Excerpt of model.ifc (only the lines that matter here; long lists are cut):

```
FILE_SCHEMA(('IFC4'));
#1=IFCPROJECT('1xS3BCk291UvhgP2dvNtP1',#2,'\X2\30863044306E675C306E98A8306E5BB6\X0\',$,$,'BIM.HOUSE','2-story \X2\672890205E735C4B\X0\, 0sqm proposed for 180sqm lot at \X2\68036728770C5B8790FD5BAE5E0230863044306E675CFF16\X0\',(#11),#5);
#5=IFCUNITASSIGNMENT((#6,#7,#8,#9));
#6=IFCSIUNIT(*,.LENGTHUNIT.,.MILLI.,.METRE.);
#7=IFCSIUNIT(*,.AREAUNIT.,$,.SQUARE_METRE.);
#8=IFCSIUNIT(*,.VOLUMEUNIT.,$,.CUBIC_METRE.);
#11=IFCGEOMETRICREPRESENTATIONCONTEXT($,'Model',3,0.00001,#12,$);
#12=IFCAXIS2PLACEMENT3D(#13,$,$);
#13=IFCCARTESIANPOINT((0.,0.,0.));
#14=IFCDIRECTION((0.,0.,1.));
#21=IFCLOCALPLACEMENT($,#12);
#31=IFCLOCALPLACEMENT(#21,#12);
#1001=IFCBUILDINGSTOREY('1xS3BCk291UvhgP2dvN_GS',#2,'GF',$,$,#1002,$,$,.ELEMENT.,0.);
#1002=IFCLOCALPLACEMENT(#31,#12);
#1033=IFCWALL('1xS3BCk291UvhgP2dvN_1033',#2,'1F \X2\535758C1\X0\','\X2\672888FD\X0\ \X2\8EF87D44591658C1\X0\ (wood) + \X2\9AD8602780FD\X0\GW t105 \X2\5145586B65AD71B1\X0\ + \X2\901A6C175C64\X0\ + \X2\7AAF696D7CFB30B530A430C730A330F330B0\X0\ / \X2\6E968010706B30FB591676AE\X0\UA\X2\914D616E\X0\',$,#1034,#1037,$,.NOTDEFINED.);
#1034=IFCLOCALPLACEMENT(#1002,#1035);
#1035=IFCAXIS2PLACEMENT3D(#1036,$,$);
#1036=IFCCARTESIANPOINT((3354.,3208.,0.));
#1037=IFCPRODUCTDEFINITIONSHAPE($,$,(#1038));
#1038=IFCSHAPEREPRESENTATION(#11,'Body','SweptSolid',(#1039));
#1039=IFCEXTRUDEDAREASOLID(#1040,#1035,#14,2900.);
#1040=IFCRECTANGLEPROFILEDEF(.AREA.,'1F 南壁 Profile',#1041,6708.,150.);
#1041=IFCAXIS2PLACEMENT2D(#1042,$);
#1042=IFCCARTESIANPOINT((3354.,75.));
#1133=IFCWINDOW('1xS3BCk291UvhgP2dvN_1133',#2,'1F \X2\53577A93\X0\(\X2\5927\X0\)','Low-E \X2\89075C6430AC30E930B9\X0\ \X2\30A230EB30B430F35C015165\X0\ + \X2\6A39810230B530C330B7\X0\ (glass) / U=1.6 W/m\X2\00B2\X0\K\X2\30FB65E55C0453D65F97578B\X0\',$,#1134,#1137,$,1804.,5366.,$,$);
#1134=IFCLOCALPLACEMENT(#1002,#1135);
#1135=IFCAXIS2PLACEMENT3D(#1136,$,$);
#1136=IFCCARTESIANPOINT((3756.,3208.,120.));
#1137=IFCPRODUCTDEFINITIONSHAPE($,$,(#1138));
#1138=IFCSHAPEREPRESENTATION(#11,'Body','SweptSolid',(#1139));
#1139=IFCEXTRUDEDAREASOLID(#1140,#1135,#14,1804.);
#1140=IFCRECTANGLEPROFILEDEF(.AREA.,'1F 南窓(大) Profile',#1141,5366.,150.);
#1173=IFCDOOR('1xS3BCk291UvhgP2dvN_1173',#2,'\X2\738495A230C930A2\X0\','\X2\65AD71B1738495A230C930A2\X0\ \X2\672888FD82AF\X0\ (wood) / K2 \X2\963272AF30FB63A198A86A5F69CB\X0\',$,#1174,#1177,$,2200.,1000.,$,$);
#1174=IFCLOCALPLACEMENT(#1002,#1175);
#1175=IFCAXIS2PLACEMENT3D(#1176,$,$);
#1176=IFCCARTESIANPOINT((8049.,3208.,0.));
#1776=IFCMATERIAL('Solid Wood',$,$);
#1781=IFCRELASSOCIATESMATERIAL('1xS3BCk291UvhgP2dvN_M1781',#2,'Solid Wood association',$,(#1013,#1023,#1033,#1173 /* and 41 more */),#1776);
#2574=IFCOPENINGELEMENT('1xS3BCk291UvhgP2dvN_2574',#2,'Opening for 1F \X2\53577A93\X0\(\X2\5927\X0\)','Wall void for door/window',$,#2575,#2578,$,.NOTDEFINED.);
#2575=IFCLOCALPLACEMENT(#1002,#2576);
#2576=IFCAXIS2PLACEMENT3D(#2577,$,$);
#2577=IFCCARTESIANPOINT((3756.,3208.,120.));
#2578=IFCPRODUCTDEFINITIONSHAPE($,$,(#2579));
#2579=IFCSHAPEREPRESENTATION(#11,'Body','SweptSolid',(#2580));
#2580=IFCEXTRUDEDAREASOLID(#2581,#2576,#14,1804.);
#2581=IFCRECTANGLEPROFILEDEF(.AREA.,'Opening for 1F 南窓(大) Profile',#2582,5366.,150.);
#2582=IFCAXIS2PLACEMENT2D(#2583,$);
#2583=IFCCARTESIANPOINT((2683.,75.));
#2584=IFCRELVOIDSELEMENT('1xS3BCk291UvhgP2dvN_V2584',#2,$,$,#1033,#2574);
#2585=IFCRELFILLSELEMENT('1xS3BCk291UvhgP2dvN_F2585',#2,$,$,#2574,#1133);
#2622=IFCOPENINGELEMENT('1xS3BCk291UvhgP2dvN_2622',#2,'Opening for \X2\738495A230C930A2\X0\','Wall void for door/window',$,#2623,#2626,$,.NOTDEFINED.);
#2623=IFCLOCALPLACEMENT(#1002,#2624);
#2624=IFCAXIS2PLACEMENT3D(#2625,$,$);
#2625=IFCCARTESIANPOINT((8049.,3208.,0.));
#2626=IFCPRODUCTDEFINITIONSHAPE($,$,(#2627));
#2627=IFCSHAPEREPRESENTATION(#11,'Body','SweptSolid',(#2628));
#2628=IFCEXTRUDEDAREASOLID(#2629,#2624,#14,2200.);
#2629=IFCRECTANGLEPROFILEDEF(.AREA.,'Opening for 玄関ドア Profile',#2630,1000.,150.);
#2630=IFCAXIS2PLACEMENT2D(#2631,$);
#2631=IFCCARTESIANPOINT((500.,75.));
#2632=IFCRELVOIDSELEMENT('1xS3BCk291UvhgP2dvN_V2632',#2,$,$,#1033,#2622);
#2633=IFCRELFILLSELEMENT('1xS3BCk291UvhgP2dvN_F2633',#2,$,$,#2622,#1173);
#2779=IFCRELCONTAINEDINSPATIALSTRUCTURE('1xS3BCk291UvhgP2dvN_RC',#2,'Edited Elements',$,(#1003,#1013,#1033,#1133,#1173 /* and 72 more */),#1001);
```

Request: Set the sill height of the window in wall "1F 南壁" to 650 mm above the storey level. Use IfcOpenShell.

```python
import numpy as np
import ifcopenshell
import ifcopenshell.api.geometry
import ifcopenshell.geom
import ifcopenshell.util.element
import ifcopenshell.util.placement
import ifcopenshell.util.shape
import ifcopenshell.util.unit

model = ifcopenshell.open("model.ifc")
unit_scale = ifcopenshell.util.unit.calculate_unit_scale(model)

window = model.by_guid("1xS3BCk291UvhgP2dvN_1133")
opening = window.FillsVoids[0].RelatingOpeningElement
storey = ifcopenshell.util.element.get_container(window, ifc_class="IfcBuildingStorey")
level = ifcopenshell.util.placement.get_local_placement(storey.ObjectPlacement)[2, 3]

# The opening's origin need not be at the sill, so measure its lowest point.
shape = ifcopenshell.geom.create_shape(ifcopenshell.geom.settings(), opening)
bottom = ifcopenshell.util.shape.get_shape_bottom_elevation(shape, shape.geometry) / unit_scale
dz = level + 0.65 / unit_scale - bottom

shift = np.array([0.0, 0.0, dz])
# The window is not placed relative to its opening, so move both.
for product in (opening, window):
    matrix = ifcopenshell.util.placement.get_local_placement(product.ObjectPlacement)
    matrix[:3, 3] += shift
    ifcopenshell.api.geometry.edit_object_placement(model, product=product, matrix=matrix, is_si=False)

print(f"moved by {dz * unit_scale:+.3f} m")

model.write("model_rev.ifc")
```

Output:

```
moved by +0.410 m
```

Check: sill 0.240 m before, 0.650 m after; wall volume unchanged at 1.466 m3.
